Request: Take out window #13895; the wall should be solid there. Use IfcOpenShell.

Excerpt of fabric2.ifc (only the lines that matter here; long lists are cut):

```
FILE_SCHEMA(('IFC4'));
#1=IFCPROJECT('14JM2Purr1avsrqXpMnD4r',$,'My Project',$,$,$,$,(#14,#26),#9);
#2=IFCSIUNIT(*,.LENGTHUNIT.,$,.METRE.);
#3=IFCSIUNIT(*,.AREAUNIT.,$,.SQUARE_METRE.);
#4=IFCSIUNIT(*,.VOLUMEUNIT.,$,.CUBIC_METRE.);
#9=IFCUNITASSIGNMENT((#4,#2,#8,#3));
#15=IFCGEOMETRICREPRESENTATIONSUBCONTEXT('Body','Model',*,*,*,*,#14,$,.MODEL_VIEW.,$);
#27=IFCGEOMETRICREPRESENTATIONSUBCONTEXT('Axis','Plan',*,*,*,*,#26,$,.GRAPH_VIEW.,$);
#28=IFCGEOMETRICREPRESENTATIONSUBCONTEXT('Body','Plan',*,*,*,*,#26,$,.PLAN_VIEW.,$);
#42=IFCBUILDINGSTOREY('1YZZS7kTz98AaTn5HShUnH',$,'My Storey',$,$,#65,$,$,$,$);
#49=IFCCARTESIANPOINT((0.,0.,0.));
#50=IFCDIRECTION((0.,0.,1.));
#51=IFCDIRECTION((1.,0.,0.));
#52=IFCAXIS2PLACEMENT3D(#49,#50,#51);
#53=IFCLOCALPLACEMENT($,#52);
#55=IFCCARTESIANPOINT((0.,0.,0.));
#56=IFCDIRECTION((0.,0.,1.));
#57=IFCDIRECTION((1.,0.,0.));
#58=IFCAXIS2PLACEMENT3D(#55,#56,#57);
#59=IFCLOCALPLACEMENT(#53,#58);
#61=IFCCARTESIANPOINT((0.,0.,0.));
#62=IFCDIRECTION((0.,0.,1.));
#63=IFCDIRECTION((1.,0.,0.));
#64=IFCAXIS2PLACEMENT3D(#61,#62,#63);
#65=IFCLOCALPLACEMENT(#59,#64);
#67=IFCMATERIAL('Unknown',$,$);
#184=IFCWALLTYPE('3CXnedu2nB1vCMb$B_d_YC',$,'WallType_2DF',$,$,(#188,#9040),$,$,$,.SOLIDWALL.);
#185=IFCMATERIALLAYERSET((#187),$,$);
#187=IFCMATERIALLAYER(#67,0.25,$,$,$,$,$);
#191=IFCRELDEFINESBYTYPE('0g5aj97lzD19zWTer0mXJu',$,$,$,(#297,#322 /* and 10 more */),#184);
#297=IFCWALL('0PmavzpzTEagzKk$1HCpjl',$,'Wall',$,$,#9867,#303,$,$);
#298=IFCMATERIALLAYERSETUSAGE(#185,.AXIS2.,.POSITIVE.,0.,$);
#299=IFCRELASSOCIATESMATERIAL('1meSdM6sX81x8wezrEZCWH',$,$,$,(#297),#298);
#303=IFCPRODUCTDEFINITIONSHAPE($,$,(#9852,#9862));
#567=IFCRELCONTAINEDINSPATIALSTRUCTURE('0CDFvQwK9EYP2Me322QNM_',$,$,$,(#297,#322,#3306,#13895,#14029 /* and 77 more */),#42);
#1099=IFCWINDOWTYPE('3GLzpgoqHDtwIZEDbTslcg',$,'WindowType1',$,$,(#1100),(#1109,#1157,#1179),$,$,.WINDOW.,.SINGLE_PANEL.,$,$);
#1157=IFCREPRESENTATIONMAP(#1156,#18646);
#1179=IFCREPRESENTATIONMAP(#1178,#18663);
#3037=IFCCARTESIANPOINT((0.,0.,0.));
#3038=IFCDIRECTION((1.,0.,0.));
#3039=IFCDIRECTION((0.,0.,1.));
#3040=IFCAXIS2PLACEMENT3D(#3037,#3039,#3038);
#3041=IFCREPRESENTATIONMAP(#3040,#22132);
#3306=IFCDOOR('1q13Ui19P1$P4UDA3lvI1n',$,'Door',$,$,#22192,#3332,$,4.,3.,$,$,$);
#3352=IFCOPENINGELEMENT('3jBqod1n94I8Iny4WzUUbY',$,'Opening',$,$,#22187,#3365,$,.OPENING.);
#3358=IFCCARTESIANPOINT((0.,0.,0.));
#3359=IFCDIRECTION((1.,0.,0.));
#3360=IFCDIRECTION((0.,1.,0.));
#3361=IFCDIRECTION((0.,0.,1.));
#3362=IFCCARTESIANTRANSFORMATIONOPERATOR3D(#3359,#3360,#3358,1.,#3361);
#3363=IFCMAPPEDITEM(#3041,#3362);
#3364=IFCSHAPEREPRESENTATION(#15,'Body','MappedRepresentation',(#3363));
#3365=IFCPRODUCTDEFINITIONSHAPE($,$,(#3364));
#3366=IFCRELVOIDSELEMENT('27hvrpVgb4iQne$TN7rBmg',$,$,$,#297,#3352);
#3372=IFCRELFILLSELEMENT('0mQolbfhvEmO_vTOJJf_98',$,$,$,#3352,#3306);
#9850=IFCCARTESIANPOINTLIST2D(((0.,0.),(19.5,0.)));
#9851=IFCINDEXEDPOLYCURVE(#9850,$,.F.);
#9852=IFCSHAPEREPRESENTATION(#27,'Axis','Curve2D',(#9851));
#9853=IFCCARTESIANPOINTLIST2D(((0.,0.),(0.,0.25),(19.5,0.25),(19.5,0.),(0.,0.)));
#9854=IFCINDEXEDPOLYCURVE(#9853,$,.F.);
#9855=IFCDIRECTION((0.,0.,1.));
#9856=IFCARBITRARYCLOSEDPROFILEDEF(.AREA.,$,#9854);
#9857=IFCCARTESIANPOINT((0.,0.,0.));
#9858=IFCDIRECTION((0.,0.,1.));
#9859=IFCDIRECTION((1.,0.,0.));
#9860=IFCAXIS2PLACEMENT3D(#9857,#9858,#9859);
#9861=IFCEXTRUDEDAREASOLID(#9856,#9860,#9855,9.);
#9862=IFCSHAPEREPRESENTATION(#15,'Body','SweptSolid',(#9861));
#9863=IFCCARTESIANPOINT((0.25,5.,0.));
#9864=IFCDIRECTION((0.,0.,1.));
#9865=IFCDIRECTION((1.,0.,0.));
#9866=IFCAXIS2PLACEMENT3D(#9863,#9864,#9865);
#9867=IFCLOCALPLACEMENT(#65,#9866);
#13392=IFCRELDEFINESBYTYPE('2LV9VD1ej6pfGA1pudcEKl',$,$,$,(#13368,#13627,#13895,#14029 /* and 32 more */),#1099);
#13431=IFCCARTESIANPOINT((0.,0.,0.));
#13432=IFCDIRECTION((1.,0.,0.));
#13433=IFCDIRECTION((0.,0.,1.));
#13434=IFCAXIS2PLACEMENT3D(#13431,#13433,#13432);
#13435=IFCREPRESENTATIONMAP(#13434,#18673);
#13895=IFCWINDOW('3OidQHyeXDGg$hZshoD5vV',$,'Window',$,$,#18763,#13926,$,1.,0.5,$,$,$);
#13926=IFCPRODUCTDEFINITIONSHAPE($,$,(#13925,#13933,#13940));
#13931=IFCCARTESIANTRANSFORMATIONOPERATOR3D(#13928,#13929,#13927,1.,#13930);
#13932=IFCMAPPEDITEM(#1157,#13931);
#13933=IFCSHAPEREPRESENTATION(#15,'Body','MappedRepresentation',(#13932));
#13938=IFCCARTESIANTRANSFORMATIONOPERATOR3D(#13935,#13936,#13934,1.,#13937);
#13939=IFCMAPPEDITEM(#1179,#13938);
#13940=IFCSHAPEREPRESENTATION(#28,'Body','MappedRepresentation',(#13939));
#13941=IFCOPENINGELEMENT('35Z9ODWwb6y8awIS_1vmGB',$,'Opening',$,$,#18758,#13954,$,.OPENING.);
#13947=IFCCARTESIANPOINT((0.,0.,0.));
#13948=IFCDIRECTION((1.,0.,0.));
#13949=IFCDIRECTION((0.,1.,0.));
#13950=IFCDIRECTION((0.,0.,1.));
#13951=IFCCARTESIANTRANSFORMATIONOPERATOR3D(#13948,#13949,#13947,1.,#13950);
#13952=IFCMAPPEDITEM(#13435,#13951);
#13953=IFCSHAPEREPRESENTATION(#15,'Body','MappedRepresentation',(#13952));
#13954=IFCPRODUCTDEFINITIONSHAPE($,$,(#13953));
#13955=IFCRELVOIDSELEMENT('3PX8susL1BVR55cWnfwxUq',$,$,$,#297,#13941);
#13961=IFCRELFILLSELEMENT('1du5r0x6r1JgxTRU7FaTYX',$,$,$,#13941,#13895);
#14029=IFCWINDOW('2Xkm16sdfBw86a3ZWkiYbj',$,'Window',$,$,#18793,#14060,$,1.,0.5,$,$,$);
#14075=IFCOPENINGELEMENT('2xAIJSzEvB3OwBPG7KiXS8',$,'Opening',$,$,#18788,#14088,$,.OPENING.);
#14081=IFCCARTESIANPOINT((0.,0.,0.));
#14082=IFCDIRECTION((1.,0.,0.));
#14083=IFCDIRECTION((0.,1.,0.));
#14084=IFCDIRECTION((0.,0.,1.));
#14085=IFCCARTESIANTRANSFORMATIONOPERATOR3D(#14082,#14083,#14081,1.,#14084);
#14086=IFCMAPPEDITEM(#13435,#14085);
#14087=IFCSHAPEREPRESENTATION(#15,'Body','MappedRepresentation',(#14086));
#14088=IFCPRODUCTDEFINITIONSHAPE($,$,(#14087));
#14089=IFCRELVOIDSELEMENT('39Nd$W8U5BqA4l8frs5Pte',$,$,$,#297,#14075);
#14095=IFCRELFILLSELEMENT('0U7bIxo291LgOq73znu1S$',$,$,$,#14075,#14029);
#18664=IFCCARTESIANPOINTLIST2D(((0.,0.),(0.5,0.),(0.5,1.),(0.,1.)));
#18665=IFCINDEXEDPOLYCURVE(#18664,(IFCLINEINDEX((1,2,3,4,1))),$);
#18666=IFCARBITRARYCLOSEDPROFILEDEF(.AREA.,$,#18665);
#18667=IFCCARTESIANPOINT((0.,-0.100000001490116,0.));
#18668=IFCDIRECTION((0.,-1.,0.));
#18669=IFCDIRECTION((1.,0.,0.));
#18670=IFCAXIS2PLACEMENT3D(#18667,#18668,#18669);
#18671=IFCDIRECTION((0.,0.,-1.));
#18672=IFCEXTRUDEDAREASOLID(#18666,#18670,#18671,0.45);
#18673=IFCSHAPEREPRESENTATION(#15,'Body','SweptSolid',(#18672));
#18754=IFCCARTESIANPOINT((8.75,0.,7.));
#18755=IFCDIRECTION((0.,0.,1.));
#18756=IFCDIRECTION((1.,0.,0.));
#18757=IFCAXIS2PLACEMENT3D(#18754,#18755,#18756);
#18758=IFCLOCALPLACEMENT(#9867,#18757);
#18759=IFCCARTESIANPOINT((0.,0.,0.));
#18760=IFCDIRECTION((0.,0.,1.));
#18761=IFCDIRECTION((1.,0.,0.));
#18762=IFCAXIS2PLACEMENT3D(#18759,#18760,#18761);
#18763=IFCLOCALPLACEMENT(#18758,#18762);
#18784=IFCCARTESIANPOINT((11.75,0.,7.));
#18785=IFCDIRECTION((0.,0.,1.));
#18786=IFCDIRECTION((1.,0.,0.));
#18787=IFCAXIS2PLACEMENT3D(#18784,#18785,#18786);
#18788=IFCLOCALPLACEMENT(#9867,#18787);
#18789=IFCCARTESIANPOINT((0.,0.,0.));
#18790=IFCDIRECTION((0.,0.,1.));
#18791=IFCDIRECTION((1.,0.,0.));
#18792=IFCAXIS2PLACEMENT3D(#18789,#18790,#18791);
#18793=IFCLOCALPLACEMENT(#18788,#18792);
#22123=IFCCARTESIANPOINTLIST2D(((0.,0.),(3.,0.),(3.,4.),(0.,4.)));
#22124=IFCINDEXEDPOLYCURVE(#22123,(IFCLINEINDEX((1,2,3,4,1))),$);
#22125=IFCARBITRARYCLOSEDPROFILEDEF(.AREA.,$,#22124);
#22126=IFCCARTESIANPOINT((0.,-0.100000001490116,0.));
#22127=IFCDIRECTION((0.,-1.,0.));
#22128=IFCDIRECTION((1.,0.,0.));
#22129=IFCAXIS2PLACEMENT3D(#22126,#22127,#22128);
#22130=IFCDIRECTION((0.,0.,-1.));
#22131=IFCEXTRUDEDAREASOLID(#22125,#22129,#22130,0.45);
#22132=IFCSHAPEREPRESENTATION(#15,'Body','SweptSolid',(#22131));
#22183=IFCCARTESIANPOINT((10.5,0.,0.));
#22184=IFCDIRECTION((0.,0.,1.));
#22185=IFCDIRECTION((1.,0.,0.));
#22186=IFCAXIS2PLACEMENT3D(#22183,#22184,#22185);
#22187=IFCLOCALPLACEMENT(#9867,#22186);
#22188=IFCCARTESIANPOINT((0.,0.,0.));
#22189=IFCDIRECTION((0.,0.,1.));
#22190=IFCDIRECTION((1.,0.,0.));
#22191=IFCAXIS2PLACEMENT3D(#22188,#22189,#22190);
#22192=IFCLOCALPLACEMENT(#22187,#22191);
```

```python
import ifcopenshell
import ifcopenshell.api.feature
import ifcopenshell.api.root
import ifcopenshell.geom
import ifcopenshell.util.shape

model = ifcopenshell.open("fabric2.ifc")
settings = ifcopenshell.geom.settings()


def volume(element):
    """Net volume in cubic metres, openings subtracted."""
    shape = ifcopenshell.geom.create_shape(settings, element)
    return ifcopenshell.util.shape.get_volume(shape.geometry)


window = model.by_id(13895)
opening = window.FillsVoids[0].RelatingOpeningElement
wall = opening.VoidsElements[0].RelatingBuildingElement
before = volume(wall)

ifcopenshell.api.root.remove_product(model, product=window)
ifcopenshell.api.feature.remove_feature(model, feature=opening)

after = volume(wall)

print(f"wall volume {before:.3f} -> {after:.3f} m3")

model.write("fabric2_rev.ifc")
```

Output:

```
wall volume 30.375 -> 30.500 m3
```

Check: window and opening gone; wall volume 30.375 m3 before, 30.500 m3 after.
